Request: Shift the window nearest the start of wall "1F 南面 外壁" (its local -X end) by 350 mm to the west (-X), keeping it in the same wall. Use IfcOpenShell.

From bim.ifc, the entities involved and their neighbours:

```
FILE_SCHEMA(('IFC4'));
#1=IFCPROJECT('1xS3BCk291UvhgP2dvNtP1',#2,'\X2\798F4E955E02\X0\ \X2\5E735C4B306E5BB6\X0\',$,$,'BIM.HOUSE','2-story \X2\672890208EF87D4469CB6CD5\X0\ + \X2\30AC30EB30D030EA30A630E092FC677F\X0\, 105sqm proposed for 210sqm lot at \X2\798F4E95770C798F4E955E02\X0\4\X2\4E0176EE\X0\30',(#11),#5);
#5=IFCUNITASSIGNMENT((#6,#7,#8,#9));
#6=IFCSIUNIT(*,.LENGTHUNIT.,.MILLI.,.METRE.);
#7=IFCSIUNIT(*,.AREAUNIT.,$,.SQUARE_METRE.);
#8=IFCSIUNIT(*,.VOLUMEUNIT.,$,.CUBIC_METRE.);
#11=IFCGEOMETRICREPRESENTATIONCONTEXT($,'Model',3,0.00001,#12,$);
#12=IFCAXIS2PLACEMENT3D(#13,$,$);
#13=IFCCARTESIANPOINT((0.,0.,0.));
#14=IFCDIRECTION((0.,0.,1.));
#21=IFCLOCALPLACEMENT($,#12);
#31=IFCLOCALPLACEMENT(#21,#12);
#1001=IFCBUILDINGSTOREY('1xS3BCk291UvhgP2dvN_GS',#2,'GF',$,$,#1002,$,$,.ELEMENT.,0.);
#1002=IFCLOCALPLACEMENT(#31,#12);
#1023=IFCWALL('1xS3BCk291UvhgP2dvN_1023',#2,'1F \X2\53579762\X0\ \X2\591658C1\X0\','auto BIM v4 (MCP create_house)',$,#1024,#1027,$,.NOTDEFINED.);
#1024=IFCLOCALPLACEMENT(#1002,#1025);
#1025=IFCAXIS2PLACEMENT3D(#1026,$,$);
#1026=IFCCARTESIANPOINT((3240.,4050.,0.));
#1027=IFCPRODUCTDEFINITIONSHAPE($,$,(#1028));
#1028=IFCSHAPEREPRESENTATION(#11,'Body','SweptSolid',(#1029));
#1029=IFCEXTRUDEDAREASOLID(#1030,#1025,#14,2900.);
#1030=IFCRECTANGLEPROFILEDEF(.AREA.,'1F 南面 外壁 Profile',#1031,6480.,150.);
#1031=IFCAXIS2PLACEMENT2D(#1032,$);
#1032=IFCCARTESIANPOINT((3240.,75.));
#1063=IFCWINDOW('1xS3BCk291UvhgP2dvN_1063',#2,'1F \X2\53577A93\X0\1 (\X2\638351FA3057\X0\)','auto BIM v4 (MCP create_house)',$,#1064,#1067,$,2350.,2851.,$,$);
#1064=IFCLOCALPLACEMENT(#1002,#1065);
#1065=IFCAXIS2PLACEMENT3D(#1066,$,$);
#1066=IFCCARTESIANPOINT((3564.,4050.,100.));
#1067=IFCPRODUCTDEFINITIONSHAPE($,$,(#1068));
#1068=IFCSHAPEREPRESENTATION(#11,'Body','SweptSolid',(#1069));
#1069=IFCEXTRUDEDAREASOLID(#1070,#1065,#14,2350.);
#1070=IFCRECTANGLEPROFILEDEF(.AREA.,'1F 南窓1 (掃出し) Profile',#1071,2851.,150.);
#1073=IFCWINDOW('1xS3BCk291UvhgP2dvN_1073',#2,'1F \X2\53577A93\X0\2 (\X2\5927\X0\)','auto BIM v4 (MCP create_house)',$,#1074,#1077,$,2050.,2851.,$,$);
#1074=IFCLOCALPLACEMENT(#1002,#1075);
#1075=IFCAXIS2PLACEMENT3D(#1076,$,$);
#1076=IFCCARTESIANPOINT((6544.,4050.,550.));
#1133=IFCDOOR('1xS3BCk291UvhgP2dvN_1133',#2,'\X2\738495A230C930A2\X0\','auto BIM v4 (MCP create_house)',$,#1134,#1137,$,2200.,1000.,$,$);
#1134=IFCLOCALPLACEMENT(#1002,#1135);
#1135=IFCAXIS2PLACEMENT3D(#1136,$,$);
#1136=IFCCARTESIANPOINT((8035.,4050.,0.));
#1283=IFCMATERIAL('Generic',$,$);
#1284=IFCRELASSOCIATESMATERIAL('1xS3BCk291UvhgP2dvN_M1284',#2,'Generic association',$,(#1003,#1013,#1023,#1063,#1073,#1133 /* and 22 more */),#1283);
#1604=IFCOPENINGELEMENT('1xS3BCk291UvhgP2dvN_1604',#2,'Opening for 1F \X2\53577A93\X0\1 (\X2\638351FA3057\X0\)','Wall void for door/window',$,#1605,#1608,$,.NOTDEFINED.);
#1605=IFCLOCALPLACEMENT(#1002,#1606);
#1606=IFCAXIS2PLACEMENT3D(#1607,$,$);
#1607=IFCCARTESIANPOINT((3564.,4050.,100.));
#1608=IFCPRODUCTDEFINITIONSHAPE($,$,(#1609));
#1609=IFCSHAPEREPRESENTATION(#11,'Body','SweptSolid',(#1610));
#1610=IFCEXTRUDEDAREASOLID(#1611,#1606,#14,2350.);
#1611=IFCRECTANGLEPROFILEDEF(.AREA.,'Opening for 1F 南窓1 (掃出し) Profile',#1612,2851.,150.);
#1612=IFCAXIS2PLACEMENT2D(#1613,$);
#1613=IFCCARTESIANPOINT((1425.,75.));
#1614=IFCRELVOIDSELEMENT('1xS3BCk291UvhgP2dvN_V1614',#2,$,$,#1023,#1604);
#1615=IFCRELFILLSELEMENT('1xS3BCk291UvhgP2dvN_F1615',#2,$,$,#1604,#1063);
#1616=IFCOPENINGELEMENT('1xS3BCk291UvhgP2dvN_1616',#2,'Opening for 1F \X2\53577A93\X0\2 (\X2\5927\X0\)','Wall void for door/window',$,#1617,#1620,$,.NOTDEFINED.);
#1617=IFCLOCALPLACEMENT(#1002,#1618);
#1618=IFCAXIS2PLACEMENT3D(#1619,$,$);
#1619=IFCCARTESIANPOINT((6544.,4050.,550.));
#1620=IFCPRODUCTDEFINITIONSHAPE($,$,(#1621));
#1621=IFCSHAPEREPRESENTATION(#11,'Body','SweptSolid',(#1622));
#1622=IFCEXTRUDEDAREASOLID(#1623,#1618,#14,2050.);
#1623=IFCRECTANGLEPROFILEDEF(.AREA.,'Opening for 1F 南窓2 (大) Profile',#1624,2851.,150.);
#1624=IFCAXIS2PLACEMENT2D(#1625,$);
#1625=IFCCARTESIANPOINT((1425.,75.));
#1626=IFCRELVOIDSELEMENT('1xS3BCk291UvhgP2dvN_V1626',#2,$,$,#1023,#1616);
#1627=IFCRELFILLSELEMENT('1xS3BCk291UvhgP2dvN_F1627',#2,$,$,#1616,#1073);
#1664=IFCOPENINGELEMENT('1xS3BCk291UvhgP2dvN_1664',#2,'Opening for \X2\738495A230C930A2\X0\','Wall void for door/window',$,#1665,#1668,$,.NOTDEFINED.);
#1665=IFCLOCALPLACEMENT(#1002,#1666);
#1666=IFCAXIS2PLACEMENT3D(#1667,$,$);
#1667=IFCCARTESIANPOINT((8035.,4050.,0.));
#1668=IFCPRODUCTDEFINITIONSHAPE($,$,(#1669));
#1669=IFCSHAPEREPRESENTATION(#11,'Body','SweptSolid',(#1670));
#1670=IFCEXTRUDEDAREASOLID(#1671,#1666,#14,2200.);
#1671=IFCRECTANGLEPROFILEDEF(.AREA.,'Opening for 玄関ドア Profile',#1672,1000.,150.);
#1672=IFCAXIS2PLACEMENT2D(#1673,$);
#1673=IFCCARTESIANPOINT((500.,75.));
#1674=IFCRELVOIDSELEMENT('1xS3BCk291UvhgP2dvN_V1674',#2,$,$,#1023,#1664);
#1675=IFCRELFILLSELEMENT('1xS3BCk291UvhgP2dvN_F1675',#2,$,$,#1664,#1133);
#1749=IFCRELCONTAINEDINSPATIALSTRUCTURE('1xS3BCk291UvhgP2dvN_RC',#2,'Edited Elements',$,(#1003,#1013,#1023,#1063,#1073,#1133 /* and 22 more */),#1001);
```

```python
import ifcopenshell
import ifcopenshell.api.geometry
import ifcopenshell.util.placement
import ifcopenshell.util.unit

model = ifcopenshell.open("bim.ifc")
unit_scale = ifcopenshell.util.unit.calculate_unit_scale(model)

window = model.by_guid("1xS3BCk291UvhgP2dvN_1063")
opening = window.FillsVoids[0].RelatingOpeningElement
wall = opening.VoidsElements[0].RelatingBuildingElement

wall_matrix = ifcopenshell.util.placement.get_local_placement(wall.ObjectPlacement)
shift = wall_matrix[:3, 0] * -0.35 / unit_scale
before = ifcopenshell.util.placement.get_local_placement(window.ObjectPlacement)[:3, 3].copy()

# The window is not placed relative to its opening, so move both.
for product in (opening, window):
    matrix = ifcopenshell.util.placement.get_local_placement(product.ObjectPlacement)
    matrix[:3, 3] += shift
    ifcopenshell.api.geometry.edit_object_placement(model, product=product, matrix=matrix, is_si=False)

after = ifcopenshell.util.placement.get_local_placement(window.ObjectPlacement)[:3, 3]
print("window moved by", (after - before).round(3) + 0.0)

model.write("bim_updated.ifc")
```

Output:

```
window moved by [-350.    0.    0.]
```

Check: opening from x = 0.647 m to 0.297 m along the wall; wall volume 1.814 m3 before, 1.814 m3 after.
